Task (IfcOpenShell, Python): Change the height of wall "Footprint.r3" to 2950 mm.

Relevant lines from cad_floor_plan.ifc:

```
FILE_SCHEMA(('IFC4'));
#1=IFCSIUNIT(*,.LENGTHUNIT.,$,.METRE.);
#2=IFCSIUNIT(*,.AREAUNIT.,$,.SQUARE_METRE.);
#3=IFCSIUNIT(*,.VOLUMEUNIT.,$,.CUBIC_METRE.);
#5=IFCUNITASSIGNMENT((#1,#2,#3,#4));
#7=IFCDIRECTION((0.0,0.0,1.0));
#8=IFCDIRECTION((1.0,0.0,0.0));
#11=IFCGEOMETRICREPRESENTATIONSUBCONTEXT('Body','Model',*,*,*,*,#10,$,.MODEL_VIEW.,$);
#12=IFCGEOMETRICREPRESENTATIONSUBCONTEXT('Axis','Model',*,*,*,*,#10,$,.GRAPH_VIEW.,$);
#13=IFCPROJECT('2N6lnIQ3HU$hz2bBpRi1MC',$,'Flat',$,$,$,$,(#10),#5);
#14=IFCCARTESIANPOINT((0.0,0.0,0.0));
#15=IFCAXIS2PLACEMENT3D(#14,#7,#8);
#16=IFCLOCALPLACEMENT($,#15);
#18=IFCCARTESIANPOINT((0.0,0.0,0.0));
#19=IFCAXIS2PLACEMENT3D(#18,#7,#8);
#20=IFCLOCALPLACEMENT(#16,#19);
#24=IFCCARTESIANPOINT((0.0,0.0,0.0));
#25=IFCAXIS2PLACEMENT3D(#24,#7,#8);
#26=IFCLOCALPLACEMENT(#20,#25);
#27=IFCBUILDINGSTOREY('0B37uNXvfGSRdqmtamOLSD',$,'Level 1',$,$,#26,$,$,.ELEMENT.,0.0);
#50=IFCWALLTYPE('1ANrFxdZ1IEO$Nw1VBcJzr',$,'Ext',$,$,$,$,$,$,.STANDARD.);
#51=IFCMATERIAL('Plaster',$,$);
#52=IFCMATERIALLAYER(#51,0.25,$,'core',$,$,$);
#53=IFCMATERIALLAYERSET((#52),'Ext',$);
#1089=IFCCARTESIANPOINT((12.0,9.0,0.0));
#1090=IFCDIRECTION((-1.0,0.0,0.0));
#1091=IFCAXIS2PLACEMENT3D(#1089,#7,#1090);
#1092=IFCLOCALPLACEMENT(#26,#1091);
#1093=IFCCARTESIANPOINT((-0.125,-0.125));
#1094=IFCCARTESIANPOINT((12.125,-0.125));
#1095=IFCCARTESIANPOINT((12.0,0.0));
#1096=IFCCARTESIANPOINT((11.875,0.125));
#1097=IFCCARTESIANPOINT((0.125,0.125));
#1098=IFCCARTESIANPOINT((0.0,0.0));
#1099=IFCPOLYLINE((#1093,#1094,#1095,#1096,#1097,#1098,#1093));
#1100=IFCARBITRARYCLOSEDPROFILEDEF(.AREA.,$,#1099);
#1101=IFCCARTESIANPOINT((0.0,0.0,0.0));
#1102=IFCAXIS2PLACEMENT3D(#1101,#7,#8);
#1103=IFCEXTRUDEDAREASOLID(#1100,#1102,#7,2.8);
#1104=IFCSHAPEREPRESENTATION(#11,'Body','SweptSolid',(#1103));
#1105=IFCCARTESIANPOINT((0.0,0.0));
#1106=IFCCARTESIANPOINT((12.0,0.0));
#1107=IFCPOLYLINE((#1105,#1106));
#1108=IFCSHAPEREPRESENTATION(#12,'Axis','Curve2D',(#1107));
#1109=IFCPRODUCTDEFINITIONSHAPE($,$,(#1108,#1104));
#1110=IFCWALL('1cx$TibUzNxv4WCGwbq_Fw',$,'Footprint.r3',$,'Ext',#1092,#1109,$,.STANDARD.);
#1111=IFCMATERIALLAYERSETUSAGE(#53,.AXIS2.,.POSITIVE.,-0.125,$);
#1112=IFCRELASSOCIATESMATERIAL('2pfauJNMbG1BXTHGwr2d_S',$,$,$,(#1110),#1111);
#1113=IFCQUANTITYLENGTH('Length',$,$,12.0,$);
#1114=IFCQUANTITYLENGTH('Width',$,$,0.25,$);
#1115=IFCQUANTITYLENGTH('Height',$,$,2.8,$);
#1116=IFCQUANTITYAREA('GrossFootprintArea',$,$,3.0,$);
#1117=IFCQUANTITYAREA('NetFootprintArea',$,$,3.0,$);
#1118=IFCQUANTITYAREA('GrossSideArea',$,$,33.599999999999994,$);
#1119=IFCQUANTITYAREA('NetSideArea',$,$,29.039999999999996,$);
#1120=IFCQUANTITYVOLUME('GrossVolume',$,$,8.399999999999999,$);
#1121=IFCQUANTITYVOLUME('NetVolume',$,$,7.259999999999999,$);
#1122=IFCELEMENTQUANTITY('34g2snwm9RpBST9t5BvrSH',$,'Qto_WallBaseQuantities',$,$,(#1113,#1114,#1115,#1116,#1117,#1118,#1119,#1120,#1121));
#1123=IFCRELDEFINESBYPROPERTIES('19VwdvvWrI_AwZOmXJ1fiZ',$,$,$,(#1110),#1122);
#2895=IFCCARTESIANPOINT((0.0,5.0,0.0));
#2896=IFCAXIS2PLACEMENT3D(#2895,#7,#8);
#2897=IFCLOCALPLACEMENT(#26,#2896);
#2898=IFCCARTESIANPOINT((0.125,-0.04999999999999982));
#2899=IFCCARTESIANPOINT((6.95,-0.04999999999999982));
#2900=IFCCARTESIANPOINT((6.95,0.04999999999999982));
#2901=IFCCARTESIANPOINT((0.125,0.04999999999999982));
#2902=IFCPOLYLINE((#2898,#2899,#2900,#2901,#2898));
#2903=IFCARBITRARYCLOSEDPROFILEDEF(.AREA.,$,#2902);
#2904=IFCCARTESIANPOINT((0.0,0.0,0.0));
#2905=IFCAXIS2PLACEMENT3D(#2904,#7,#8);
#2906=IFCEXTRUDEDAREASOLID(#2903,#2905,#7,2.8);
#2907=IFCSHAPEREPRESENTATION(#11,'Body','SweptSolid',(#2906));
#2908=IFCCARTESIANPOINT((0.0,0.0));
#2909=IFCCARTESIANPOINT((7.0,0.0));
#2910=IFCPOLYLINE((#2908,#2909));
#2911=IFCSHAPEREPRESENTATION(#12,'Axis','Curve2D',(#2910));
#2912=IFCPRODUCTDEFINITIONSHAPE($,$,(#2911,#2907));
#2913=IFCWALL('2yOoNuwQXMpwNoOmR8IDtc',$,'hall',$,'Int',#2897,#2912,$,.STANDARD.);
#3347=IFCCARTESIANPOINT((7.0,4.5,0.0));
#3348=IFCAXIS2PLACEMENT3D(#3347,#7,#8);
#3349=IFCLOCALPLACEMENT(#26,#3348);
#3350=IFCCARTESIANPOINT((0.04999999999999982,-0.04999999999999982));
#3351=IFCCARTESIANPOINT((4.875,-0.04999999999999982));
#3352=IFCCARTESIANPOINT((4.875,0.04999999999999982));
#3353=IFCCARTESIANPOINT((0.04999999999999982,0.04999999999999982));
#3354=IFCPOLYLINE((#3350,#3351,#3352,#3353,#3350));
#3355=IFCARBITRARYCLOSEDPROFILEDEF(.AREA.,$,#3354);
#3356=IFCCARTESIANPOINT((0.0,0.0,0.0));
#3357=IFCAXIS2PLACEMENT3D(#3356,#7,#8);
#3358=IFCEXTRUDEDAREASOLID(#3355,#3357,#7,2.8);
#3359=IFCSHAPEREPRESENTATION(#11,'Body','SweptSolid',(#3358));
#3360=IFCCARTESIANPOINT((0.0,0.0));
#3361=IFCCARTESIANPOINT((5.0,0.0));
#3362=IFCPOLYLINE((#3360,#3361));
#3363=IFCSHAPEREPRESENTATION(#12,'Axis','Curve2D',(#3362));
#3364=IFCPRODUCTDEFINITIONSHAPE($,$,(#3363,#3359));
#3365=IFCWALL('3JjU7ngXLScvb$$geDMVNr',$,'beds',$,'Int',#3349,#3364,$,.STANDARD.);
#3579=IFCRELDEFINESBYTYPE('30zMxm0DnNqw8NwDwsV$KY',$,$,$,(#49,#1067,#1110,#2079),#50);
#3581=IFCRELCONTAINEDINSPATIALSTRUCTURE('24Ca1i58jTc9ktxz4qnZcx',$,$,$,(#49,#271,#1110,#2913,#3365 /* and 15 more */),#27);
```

```python
import ifcopenshell
import ifcopenshell.api.pset
import ifcopenshell.geom
import ifcopenshell.util.element
import ifcopenshell.util.representation
import ifcopenshell.util.shape
import ifcopenshell.util.unit

model = ifcopenshell.open("cad_floor_plan.ifc")
unit_scale = ifcopenshell.util.unit.calculate_unit_scale(model)
area_scale = ifcopenshell.util.unit.calculate_unit_scale(model, "AREAUNIT")
volume_scale = ifcopenshell.util.unit.calculate_unit_scale(model, "VOLUMEUNIT")
settings = ifcopenshell.geom.settings()


def volume(element):
    """Net volume in cubic metres, openings subtracted."""
    shape = ifcopenshell.geom.create_shape(settings, element)
    return ifcopenshell.util.shape.get_volume(shape.geometry)


wall = model.by_guid("1cx$TibUzNxv4WCGwbq_Fw")
before = volume(wall)

body = ifcopenshell.util.representation.get_representation(wall, "Model", "Body")
solid = body.Items[0]
old_height = solid.Depth
solid.Depth = 2.95
after = volume(wall)
thickness = 0.25  # wall thickness in metres

# Update the stored height, areas and volumes.
qto = model.by_id(ifcopenshell.util.element.get_pset(wall, "Qto_WallBaseQuantities", should_inherit=False)["id"])
ifcopenshell.api.pset.edit_qto(model, qto=qto, properties={
    "Height": solid.Depth,
    "GrossSideArea": ifcopenshell.util.element.get_pset(wall, "Qto_WallBaseQuantities", "GrossSideArea") * solid.Depth / old_height,
    "NetSideArea": after / thickness / area_scale,
    "GrossVolume": ifcopenshell.util.element.get_pset(wall, "Qto_WallBaseQuantities", "GrossVolume") * solid.Depth / old_height,
    "NetVolume": after / volume_scale,
})

print(f"height {old_height:g} -> {solid.Depth:g}, volume {before:.3f} -> {after:.3f} m3")

model.write("cad_floor_plan_v2.ifc")
```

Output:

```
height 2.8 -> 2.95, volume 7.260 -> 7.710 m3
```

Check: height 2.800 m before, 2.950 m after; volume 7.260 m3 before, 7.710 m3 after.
